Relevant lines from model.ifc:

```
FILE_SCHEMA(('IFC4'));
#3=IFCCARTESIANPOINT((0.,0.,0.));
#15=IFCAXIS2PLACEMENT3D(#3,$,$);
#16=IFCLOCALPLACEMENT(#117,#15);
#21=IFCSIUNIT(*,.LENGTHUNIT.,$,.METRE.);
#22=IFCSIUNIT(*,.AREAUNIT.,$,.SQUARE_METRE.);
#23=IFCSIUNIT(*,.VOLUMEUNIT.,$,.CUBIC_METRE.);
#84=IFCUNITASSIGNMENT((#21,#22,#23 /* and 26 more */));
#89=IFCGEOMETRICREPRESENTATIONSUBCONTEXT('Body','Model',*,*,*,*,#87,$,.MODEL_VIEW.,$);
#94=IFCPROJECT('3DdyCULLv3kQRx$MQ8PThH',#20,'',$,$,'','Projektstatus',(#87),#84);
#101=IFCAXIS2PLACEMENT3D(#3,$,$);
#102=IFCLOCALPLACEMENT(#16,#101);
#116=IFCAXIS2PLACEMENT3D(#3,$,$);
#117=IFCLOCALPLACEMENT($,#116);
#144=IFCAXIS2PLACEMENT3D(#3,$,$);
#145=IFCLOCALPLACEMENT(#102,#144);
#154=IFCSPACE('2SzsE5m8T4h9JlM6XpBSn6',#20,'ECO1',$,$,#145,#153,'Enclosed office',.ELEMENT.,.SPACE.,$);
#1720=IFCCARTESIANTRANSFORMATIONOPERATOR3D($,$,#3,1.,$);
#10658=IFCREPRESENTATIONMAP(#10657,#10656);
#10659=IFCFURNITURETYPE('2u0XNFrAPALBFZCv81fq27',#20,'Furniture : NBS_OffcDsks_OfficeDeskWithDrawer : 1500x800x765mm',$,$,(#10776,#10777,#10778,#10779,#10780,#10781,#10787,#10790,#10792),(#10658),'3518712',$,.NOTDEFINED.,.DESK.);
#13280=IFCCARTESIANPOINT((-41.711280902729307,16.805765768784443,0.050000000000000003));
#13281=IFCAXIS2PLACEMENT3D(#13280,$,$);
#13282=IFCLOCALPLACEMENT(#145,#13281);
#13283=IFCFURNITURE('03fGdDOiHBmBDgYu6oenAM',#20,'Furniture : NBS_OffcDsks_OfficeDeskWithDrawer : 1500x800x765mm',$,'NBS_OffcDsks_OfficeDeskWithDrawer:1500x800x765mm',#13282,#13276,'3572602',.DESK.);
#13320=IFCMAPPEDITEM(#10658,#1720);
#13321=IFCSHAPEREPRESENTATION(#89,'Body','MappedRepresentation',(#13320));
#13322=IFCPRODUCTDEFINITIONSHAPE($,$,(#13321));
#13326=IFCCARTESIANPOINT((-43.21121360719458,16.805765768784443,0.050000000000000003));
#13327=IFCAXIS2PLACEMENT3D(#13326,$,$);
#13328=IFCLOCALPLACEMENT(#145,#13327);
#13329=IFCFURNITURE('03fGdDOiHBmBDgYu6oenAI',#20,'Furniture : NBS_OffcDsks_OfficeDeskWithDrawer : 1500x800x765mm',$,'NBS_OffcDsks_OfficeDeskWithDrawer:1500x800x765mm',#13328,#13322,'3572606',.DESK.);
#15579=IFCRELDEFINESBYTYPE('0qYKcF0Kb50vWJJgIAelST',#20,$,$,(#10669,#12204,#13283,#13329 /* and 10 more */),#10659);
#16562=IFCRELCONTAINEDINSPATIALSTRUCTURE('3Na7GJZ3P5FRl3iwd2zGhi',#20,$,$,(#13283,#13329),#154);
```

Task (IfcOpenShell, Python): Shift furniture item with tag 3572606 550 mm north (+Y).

```python
import ifcopenshell
import ifcopenshell.api.geometry
import ifcopenshell.util.placement

model = ifcopenshell.open("model.ifc")

item = model.by_guid("03fGdDOiHBmBDgYu6oenAI")
matrix = ifcopenshell.util.placement.get_local_placement(item.ObjectPlacement)
matrix[1, 3] += 0.55
ifcopenshell.api.geometry.edit_object_placement(model, product=item, matrix=matrix, is_si=False)

print(ifcopenshell.util.placement.get_local_placement(item.ObjectPlacement).round(3) + 0.0)

model.write("model-out.ifc")
```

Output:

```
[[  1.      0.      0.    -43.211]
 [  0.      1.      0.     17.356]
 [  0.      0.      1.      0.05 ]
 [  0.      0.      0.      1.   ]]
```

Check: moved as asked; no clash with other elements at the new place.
